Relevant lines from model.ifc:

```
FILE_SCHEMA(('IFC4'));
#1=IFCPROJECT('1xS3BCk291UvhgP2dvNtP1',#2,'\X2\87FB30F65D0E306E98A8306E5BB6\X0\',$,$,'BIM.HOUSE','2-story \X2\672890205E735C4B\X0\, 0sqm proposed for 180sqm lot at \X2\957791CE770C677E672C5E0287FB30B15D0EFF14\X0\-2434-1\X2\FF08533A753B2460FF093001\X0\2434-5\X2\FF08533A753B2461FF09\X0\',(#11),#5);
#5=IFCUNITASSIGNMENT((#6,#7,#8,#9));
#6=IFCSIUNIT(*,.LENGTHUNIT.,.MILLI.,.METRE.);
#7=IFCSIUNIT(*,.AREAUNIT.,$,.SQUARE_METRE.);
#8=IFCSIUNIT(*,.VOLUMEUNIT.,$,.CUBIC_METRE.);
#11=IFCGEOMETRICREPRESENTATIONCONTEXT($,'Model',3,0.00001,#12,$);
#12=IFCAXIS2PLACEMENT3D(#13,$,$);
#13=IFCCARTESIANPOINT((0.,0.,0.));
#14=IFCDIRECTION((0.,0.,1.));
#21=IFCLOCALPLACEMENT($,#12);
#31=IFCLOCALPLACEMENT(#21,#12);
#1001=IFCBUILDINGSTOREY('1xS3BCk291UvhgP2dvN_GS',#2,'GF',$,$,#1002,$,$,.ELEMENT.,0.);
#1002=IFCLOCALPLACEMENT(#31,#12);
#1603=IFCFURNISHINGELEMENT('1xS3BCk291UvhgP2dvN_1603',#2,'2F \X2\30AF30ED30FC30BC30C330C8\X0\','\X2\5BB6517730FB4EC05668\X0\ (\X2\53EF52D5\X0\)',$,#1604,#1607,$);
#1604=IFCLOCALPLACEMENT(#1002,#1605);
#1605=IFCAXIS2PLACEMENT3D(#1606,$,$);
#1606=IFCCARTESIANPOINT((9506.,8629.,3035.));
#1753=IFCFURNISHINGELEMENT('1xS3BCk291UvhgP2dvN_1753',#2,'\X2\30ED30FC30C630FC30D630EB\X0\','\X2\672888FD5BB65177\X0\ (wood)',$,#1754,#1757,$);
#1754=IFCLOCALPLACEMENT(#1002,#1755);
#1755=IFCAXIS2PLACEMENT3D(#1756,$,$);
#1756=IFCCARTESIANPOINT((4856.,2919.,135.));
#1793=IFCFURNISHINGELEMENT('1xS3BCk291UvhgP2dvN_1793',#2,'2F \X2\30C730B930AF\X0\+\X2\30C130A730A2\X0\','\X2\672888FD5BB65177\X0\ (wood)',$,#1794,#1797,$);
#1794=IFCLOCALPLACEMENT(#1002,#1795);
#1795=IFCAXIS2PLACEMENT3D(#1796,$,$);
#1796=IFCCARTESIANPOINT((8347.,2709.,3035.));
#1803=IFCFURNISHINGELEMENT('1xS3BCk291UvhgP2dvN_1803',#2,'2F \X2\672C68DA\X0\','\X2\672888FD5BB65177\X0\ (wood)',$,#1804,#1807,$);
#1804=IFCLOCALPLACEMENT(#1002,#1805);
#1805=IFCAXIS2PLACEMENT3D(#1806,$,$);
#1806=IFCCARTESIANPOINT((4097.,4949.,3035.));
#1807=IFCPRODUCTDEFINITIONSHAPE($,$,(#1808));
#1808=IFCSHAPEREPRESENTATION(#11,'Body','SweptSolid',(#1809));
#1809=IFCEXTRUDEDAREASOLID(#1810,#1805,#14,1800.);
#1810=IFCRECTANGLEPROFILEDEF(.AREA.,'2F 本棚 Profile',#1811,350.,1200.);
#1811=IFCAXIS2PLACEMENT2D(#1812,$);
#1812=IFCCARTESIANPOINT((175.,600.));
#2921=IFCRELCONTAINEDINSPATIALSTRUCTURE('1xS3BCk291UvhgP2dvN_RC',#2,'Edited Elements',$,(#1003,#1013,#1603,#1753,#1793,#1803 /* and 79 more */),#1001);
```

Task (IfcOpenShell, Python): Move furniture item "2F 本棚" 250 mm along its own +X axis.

```python
import ifcopenshell
import ifcopenshell.api.geometry
import ifcopenshell.util.placement
import ifcopenshell.util.unit

model = ifcopenshell.open("model.ifc")
unit_scale = ifcopenshell.util.unit.calculate_unit_scale(model)

item = model.by_id(1803)
matrix = ifcopenshell.util.placement.get_local_placement(item.ObjectPlacement)
matrix[:3, 3] += matrix[:3, 0] * 0.25 / unit_scale
ifcopenshell.api.geometry.edit_object_placement(model, product=item, matrix=matrix, is_si=False)

print(ifcopenshell.util.placement.get_local_placement(item.ObjectPlacement).round(3) + 0.0)

model.write("model_updated.ifc")
```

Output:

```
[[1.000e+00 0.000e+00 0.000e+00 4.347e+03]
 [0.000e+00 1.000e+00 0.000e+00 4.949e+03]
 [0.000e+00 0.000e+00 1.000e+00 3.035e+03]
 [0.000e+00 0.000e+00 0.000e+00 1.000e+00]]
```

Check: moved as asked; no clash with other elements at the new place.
